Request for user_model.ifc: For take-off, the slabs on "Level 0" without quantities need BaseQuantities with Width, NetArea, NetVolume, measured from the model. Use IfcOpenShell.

First a look at what the model holds.

```python
import ifcopenshell
import ifcopenshell.util.element
import ifcopenshell.util.unit

model = ifcopenshell.open("user_model.ifc")
print(model.schema)
for unit_type in ("LENGTHUNIT", "AREAUNIT", "VOLUMEUNIT"):
    print(unit_type, ifcopenshell.util.unit.calculate_unit_scale(model, unit_type))
storey = next(s for s in model.by_type("IfcBuildingStorey") if s.Name == "Level 0")
slabs = [e for e in ifcopenshell.util.element.get_decomposition(storey) if e.is_a("IfcSlab")]
for e in sorted(slabs, key=lambda e: e.id()):
    print(e.id(), e.is_a(), e.Name, list(ifcopenshell.util.element.get_psets(e, qtos_only=True)), sep=" | ")
```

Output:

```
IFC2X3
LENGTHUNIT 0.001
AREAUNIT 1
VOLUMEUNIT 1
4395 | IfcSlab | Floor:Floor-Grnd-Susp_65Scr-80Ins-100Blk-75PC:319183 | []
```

```python
import ifcopenshell
import ifcopenshell.api.pset
import ifcopenshell.geom
import ifcopenshell.util.element
import ifcopenshell.util.shape
import ifcopenshell.util.unit

model = ifcopenshell.open("user_model.ifc")
unit_scale = ifcopenshell.util.unit.calculate_unit_scale(model)
area_scale = ifcopenshell.util.unit.calculate_unit_scale(model, "AREAUNIT")
volume_scale = ifcopenshell.util.unit.calculate_unit_scale(model, "VOLUMEUNIT")
settings = ifcopenshell.geom.settings()

storey = next(s for s in model.by_type("IfcBuildingStorey") if s.Name == "Level 0")
slabs = [e for e in ifcopenshell.util.element.get_decomposition(storey) if e.is_a("IfcSlab")]

for e in sorted(slabs, key=lambda e: e.id()):
    if ifcopenshell.util.element.get_psets(e, qtos_only=True, should_inherit=False):
        continue
    # Geometry comes back in metres, in the element's own axes.
    shape = ifcopenshell.geom.create_shape(settings, e)
    values = {
        "Width": ifcopenshell.util.shape.get_z(shape.geometry) / unit_scale,
        "NetArea": ifcopenshell.util.shape.get_footprint_area(shape.geometry) / area_scale,
        "NetVolume": ifcopenshell.util.shape.get_volume(shape.geometry) / volume_scale,
    }
    qto = ifcopenshell.api.pset.add_qto(model, product=e, name="BaseQuantities")
    ifcopenshell.api.pset.edit_qto(model, qto=qto, properties=values)
    print(e.id(), {k: round(v, 3) for k, v in values.items()})

model.write("user_model_edited.ifc")
```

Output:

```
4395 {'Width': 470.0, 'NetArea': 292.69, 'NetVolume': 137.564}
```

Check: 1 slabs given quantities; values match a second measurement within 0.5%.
